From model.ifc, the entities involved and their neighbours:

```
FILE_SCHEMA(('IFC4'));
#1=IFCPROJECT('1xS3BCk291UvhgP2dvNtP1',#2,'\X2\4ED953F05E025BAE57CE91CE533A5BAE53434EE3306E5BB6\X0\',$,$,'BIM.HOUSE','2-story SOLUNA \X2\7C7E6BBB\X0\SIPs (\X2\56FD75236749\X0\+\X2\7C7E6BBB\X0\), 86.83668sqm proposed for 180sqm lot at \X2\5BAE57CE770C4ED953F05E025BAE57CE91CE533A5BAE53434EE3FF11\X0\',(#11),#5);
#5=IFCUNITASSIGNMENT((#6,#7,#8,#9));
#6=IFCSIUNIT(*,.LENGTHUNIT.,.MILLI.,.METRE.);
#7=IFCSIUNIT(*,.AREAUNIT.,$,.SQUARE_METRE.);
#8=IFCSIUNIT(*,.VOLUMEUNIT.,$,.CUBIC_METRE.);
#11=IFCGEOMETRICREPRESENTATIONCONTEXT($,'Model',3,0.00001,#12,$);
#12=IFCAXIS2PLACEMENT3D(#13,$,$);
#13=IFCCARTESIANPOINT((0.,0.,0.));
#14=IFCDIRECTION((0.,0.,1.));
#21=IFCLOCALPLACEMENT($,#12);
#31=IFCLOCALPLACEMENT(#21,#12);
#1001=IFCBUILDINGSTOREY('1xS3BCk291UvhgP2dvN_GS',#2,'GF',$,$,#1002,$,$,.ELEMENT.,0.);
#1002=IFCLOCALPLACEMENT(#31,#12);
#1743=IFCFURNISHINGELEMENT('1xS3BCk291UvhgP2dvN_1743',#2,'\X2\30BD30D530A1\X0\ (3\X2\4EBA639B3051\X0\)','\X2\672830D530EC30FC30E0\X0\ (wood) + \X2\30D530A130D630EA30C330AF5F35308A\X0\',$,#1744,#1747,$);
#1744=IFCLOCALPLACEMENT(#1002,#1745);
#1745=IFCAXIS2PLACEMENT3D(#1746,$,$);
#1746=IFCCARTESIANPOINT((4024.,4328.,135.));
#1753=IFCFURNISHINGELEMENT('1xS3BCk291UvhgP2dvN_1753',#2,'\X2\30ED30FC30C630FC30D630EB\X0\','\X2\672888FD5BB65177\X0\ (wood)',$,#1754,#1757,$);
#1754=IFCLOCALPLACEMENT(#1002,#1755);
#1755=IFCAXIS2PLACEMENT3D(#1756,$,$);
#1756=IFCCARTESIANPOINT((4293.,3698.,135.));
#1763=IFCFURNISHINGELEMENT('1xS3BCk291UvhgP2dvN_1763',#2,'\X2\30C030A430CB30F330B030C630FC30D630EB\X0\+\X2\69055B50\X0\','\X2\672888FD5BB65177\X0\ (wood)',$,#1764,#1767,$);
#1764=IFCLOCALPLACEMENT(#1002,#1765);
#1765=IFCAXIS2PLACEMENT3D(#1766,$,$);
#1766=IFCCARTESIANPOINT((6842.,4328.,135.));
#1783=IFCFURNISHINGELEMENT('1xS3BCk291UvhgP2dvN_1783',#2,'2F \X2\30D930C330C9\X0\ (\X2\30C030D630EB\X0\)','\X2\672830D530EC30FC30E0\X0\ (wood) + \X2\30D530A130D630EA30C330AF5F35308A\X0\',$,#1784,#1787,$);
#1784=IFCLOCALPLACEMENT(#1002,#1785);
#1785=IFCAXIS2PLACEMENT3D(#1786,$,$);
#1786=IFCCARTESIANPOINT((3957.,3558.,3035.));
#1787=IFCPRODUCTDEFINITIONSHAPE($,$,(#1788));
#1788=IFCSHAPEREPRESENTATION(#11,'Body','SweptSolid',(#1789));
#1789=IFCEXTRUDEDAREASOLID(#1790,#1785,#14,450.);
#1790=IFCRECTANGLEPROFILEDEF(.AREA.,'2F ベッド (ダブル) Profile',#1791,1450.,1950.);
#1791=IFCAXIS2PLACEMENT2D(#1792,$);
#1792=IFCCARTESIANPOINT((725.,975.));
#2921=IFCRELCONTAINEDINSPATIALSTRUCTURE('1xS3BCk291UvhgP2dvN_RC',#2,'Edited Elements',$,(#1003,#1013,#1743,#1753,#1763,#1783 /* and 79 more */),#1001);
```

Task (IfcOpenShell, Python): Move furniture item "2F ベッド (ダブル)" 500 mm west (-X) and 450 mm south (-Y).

```python
import ifcopenshell
import ifcopenshell.api.geometry
import ifcopenshell.util.placement
import ifcopenshell.util.unit

model = ifcopenshell.open("model.ifc")
unit_scale = ifcopenshell.util.unit.calculate_unit_scale(model)

item = model.by_guid("1xS3BCk291UvhgP2dvN_1783")
matrix = ifcopenshell.util.placement.get_local_placement(item.ObjectPlacement)
matrix[0, 3] -= 0.5 / unit_scale
matrix[1, 3] -= 0.45 / unit_scale
ifcopenshell.api.geometry.edit_object_placement(model, product=item, matrix=matrix, is_si=False)

print(ifcopenshell.util.placement.get_local_placement(item.ObjectPlacement).round(3) + 0.0)

model.write("model_v2.ifc")
```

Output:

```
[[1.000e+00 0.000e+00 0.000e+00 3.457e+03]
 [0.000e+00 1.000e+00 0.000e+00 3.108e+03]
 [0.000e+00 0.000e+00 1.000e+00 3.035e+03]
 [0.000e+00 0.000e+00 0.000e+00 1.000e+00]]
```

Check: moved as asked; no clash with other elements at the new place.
